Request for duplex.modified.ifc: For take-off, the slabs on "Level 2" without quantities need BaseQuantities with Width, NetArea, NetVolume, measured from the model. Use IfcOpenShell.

First a look at what the model holds.

```python
import ifcopenshell
import ifcopenshell.util.element
import ifcopenshell.util.unit

model = ifcopenshell.open("duplex.modified.ifc")
print(model.schema)
for unit_type in ("LENGTHUNIT", "AREAUNIT", "VOLUMEUNIT"):
    print(unit_type, ifcopenshell.util.unit.calculate_unit_scale(model, unit_type))
storey = next(s for s in model.by_type("IfcBuildingStorey") if s.Name == "Level 2")
slabs = [e for e in ifcopenshell.util.element.get_decomposition(storey) if e.is_a("IfcSlab")]
for e in sorted(slabs, key=lambda e: e.id()):
    print(e.id(), e.is_a(), e.Name, list(ifcopenshell.util.element.get_psets(e, qtos_only=True)), sep=" | ")
```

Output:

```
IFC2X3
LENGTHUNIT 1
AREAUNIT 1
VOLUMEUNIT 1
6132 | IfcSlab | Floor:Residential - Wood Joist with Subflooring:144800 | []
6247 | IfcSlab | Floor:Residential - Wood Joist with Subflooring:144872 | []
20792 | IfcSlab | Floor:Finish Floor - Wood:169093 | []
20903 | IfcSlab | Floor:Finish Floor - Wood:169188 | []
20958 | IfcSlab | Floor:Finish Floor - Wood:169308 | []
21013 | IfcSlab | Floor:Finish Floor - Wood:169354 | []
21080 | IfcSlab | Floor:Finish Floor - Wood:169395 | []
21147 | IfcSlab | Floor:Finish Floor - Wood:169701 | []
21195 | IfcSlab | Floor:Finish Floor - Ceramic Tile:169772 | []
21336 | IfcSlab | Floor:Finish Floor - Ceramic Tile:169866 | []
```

```python
import ifcopenshell
import ifcopenshell.api.pset
import ifcopenshell.geom
import ifcopenshell.util.element
import ifcopenshell.util.shape
import ifcopenshell.util.unit

model = ifcopenshell.open("duplex.modified.ifc")
unit_scale = ifcopenshell.util.unit.calculate_unit_scale(model)
area_scale = ifcopenshell.util.unit.calculate_unit_scale(model, "AREAUNIT")
volume_scale = ifcopenshell.util.unit.calculate_unit_scale(model, "VOLUMEUNIT")
settings = ifcopenshell.geom.settings()

storey = next(s for s in model.by_type("IfcBuildingStorey") if s.Name == "Level 2")
slabs = [e for e in ifcopenshell.util.element.get_decomposition(storey) if e.is_a("IfcSlab")]

for e in sorted(slabs, key=lambda e: e.id()):
    if ifcopenshell.util.element.get_psets(e, qtos_only=True, should_inherit=False):
        continue
    # Geometry comes back in metres, in the element's own axes.
    shape = ifcopenshell.geom.create_shape(settings, e)
    values = {
        "Width": ifcopenshell.util.shape.get_z(shape.geometry) / unit_scale,
        "NetArea": ifcopenshell.util.shape.get_footprint_area(shape.geometry) / area_scale,
        "NetVolume": ifcopenshell.util.shape.get_volume(shape.geometry) / volume_scale,
    }
    qto = ifcopenshell.api.pset.add_qto(model, product=e, name="BaseQuantities")
    ifcopenshell.api.pset.edit_qto(model, qto=qto, properties=values)
    print(e.id(), {k: round(v, 3) for k, v in values.items()})

model.write("duplex.modified_rev.ifc")
```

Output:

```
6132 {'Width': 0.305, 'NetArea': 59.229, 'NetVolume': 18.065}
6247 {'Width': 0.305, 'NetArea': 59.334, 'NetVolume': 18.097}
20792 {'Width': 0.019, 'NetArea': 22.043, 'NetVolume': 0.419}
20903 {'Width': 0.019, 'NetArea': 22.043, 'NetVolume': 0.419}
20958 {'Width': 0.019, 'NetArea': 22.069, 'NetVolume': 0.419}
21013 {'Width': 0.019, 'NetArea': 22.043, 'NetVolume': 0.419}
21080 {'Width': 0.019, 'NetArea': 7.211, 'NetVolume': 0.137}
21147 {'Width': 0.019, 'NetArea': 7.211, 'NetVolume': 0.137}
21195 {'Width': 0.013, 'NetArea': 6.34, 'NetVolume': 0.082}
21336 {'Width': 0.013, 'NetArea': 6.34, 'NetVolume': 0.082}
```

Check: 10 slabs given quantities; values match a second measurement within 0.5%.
